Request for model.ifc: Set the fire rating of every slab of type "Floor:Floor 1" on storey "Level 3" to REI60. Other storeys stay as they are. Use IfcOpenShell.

First a look at what the model holds.

```python
import ifcopenshell
import ifcopenshell.util.element

model = ifcopenshell.open("model.ifc")
print(model.schema)
storey = next(s for s in model.by_type("IfcBuildingStorey") if s.Name == "Level 3")
slabs = [e for e in ifcopenshell.util.element.get_decomposition(storey) if e.is_a("IfcSlab")]
seen = {}
for e in slabs:
    element_type = ifcopenshell.util.element.get_type(e)
    key = (element_type.Name if element_type != e and element_type else None, ifcopenshell.util.element.get_pset(e, "Pset_SlabCommon", "FireRating"))
    seen[key] = seen.get(key, 0) + 1
for (name, value), count in sorted(seen.items(), key=str):
    print(count, "x", name, "|", value)
```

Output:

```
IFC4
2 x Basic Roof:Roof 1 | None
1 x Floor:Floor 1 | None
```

```python
import ifcopenshell
import ifcopenshell.api.pset
import ifcopenshell.util.element

model = ifcopenshell.open("model.ifc")

storey = next(s for s in model.by_type("IfcBuildingStorey") if s.Name == "Level 3")
slabs = [e for e in ifcopenshell.util.element.get_decomposition(storey) if e.is_a("IfcSlab")]

count = 0
for e in slabs:
    element_type = ifcopenshell.util.element.get_type(e)
    if element_type in (None, e) or element_type.Name != "Floor:Floor 1":
        continue
    # add_pset returns the element's existing set when there is one.
    pset = ifcopenshell.api.pset.add_pset(model, product=e, name="Pset_SlabCommon")
    ifcopenshell.api.pset.edit_pset(model, pset=pset, properties={"FireRating": "REI60"})
    count += 1

print(count, "slabs updated")

model.write("model-out.ifc")
```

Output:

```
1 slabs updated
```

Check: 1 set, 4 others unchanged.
